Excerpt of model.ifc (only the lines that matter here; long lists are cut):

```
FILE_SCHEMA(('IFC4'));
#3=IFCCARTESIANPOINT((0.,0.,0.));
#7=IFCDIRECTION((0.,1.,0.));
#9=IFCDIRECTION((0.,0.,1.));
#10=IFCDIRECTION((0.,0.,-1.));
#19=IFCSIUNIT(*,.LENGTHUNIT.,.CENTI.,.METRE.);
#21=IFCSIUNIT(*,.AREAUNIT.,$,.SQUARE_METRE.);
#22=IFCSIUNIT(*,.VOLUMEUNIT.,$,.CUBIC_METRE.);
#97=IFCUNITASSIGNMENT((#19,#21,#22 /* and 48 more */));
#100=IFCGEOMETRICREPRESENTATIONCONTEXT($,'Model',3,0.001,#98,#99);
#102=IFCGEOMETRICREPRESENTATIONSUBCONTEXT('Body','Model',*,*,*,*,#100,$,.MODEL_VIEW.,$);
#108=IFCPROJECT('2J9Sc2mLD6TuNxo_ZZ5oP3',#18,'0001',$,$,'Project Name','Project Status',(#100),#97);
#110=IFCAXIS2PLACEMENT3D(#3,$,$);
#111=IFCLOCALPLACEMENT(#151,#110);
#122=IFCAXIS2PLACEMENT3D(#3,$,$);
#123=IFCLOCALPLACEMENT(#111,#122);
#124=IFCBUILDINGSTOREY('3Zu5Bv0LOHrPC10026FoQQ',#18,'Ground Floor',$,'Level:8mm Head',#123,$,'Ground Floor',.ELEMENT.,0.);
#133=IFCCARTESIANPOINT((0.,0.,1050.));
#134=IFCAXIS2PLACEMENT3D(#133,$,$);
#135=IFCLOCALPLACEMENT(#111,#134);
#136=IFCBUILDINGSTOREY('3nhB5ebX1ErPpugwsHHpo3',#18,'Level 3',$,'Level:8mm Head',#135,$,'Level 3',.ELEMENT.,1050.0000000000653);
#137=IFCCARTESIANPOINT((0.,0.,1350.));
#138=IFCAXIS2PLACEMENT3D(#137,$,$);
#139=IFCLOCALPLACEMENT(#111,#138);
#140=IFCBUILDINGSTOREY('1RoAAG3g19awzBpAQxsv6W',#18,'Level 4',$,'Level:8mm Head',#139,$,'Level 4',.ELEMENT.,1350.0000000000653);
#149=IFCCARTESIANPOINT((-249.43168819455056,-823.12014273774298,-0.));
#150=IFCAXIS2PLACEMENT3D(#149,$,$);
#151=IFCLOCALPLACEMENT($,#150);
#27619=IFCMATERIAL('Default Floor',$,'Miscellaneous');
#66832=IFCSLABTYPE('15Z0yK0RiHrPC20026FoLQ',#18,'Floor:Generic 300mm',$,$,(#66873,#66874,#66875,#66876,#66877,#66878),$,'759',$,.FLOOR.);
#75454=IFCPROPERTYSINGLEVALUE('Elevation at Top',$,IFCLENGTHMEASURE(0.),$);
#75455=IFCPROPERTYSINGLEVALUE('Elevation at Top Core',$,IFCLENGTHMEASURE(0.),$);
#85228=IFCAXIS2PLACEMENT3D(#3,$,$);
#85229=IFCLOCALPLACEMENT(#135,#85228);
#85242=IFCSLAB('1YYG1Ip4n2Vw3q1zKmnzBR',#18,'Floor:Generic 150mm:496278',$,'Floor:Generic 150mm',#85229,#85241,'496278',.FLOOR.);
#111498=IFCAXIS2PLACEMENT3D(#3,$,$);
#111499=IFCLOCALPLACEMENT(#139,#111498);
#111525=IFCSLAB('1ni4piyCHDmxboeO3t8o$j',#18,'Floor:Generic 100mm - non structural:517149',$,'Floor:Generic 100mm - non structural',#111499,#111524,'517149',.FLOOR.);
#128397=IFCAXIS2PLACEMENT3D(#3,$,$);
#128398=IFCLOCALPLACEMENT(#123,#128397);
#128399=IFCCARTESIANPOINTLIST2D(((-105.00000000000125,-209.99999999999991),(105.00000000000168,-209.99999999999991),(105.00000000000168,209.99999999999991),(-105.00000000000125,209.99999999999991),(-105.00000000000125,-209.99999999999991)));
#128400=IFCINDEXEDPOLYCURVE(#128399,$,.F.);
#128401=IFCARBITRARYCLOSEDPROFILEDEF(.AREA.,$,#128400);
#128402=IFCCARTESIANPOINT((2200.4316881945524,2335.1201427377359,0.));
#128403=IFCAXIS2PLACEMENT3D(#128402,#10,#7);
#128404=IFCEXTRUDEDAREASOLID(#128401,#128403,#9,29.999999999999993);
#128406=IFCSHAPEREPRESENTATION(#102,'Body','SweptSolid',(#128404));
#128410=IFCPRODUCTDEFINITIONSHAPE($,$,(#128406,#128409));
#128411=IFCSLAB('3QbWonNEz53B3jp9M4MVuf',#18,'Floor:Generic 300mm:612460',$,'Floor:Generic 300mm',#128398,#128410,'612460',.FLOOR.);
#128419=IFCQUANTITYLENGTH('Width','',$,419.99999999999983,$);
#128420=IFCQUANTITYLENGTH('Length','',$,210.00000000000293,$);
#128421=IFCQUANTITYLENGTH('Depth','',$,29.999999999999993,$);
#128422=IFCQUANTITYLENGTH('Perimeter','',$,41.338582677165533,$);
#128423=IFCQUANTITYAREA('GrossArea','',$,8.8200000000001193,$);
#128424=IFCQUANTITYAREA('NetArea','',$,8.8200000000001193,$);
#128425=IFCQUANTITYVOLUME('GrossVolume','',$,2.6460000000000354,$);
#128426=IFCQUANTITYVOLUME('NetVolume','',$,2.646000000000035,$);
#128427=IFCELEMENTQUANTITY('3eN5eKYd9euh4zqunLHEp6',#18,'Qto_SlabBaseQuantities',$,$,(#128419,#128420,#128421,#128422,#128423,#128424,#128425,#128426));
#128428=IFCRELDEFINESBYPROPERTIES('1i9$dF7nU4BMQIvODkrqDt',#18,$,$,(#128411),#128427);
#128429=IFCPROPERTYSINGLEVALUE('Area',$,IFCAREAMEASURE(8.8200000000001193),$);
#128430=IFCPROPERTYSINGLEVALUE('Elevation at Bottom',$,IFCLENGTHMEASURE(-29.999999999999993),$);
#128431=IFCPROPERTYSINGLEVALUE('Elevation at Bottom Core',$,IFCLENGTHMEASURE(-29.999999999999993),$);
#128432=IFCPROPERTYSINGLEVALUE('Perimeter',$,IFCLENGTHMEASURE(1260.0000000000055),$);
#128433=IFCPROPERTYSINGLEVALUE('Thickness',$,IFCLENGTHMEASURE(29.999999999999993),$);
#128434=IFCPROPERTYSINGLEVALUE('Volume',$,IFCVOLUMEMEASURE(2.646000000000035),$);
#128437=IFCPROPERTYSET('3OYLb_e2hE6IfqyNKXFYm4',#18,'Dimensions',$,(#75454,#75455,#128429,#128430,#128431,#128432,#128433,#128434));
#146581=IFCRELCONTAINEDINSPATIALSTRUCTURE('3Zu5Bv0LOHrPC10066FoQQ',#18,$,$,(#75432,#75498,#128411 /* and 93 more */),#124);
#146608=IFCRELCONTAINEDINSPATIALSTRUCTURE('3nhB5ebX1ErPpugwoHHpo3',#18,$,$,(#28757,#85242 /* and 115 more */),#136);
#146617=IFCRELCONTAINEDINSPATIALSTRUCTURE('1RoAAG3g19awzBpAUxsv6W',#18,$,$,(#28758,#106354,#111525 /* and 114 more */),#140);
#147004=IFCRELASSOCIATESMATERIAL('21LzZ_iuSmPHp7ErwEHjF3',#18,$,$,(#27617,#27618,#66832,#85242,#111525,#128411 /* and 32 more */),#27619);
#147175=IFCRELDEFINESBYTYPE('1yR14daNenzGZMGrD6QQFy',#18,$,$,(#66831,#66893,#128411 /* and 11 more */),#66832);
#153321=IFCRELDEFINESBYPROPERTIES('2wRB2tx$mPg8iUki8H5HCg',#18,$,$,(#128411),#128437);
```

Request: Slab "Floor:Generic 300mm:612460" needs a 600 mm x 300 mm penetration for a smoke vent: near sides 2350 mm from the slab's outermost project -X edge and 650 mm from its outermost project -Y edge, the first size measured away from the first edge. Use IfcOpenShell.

```python
import numpy as np
import ifcopenshell
import ifcopenshell.api.feature
import ifcopenshell.api.geometry
import ifcopenshell.api.pset
import ifcopenshell.api.root
import ifcopenshell.geom
import ifcopenshell.util.element
import ifcopenshell.util.placement
import ifcopenshell.util.representation
import ifcopenshell.util.shape
import ifcopenshell.util.unit

model = ifcopenshell.open("model.ifc")
unit_scale = ifcopenshell.util.unit.calculate_unit_scale(model)
area_scale = ifcopenshell.util.unit.calculate_unit_scale(model, "AREAUNIT")
volume_scale = ifcopenshell.util.unit.calculate_unit_scale(model, "VOLUMEUNIT")
settings = ifcopenshell.geom.settings()


def volume(element):
    """Net volume in cubic metres, openings subtracted."""
    shape = ifcopenshell.geom.create_shape(settings, element)
    return ifcopenshell.util.shape.get_volume(shape.geometry)


slab = model.by_id(128411)
before = volume(slab)

# Extent in the slab's own axes, in metres. The edges named are its -X and -Y sides.
slab_shape = ifcopenshell.geom.create_shape(settings, slab)
vertices = ifcopenshell.util.shape.get_vertices(slab_shape.geometry)
x_min, y_min, bottom = vertices.min(axis=0)
top = vertices[:, 2].max()

opening = ifcopenshell.api.root.create_entity(model, ifc_class="IfcOpeningElement", name="Smoke vent opening", predefined_type="OPENING")
context = ifcopenshell.util.representation.get_context(model, "Model", "Body", "MODEL_VIEW")
width, depth = 0.6, 0.3
outline = [(0.0, 0.0), (width, 0.0), (width, depth), (0.0, depth), (0.0, 0.0)]
# Overshoot both faces by 50 mm so the cut is clean.
shape = ifcopenshell.api.geometry.add_slab_representation(
    model, context=context, depth=top - bottom + 0.1, polyline=outline
)
ifcopenshell.api.geometry.assign_representation(model, product=opening, representation=shape)

matrix = ifcopenshell.util.placement.get_local_placement(slab.ObjectPlacement)
matrix[:, 3] = matrix @ np.append(np.array([x_min + 2.35, y_min + 0.65, bottom - 0.05]) / unit_scale, 1.0)
ifcopenshell.api.geometry.edit_object_placement(model, product=opening, matrix=matrix, is_si=False)
ifcopenshell.api.feature.add_feature(model, feature=opening, element=slab)

after = volume(slab)

# Update the slab's stored quantities.
qto = model.by_id(ifcopenshell.util.element.get_pset(slab, "Qto_SlabBaseQuantities", should_inherit=False)["id"])
ifcopenshell.api.pset.edit_qto(model, qto=qto, properties={
    "NetArea": after / (top - bottom) / area_scale,
    "NetVolume": after / volume_scale,
})
pset = model.by_id(ifcopenshell.util.element.get_pset(slab, "Dimensions", should_inherit=False)["id"])
ifcopenshell.api.pset.edit_pset(model, pset=pset, properties={
    "Area": model.create_entity("IfcAreaMeasure", after / (top - bottom) / area_scale),
    "Volume": model.create_entity("IfcVolumeMeasure", after / volume_scale),
})

print(f"slab volume {before:.3f} -> {after:.3f} m3")

model.write("model_updated.ifc")
```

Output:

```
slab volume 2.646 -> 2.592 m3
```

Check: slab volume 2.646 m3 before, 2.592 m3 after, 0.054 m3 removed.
